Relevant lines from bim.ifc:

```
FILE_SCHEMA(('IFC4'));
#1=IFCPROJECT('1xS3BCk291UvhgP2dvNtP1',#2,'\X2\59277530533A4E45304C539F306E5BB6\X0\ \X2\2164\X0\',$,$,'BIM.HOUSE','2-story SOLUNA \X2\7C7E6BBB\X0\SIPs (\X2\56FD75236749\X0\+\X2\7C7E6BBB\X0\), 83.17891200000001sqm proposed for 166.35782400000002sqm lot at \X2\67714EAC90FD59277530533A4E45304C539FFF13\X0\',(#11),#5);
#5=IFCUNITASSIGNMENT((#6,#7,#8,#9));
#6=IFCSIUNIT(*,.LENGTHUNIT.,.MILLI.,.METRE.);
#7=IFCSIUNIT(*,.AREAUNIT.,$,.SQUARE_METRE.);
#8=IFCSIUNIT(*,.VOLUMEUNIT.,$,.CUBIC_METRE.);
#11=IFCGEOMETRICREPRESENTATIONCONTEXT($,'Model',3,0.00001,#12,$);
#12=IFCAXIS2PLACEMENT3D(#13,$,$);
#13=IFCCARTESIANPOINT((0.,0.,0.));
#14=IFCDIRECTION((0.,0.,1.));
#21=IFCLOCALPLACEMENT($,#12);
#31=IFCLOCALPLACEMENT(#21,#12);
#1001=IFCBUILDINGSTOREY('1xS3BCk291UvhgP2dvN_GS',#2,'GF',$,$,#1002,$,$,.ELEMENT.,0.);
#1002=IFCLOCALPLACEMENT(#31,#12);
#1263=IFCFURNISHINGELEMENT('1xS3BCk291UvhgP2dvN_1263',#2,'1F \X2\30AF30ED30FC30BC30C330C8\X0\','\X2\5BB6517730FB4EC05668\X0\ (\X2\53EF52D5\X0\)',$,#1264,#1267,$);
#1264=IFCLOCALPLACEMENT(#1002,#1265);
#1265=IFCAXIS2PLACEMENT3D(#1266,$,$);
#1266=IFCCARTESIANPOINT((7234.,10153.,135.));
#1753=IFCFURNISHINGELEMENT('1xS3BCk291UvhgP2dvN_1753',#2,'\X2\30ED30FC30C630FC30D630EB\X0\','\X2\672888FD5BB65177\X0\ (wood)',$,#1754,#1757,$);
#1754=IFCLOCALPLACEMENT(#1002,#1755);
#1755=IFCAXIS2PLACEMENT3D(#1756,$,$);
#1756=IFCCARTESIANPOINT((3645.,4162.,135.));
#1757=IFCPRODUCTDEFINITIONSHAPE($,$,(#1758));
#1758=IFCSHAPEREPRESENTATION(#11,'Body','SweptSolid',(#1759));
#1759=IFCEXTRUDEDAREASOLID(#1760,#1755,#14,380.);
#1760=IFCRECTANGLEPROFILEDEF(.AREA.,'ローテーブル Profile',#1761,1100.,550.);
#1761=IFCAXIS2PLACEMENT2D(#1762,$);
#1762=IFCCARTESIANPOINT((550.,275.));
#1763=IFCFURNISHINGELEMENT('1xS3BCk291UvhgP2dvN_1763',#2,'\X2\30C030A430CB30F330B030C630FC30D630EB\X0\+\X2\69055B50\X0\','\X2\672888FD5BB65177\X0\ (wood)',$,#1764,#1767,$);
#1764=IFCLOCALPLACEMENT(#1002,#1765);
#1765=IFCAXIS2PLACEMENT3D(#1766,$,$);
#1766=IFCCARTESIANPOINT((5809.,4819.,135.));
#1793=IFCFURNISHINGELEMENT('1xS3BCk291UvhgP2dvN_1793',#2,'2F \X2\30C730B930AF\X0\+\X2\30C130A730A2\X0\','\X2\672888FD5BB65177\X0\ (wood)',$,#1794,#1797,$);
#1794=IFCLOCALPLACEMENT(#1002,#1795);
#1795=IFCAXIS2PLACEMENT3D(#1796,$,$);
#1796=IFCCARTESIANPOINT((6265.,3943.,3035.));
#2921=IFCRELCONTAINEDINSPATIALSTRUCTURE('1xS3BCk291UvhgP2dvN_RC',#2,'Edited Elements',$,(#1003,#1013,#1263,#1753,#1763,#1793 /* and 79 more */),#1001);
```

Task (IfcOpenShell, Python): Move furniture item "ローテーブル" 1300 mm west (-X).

```python
import ifcopenshell
import ifcopenshell.api.geometry
import ifcopenshell.util.placement

model = ifcopenshell.open("bim.ifc")

item = model.by_id(1753)
matrix = ifcopenshell.util.placement.get_local_placement(item.ObjectPlacement)
matrix[0, 3] -= 1300.0
ifcopenshell.api.geometry.edit_object_placement(model, product=item, matrix=matrix, is_si=False)

print(ifcopenshell.util.placement.get_local_placement(item.ObjectPlacement).round(3) + 0.0)

model.write("bim_v2.ifc")
```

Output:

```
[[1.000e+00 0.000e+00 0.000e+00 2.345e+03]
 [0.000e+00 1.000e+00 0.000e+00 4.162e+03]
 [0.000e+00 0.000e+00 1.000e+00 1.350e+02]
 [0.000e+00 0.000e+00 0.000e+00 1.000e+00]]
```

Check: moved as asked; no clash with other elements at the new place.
